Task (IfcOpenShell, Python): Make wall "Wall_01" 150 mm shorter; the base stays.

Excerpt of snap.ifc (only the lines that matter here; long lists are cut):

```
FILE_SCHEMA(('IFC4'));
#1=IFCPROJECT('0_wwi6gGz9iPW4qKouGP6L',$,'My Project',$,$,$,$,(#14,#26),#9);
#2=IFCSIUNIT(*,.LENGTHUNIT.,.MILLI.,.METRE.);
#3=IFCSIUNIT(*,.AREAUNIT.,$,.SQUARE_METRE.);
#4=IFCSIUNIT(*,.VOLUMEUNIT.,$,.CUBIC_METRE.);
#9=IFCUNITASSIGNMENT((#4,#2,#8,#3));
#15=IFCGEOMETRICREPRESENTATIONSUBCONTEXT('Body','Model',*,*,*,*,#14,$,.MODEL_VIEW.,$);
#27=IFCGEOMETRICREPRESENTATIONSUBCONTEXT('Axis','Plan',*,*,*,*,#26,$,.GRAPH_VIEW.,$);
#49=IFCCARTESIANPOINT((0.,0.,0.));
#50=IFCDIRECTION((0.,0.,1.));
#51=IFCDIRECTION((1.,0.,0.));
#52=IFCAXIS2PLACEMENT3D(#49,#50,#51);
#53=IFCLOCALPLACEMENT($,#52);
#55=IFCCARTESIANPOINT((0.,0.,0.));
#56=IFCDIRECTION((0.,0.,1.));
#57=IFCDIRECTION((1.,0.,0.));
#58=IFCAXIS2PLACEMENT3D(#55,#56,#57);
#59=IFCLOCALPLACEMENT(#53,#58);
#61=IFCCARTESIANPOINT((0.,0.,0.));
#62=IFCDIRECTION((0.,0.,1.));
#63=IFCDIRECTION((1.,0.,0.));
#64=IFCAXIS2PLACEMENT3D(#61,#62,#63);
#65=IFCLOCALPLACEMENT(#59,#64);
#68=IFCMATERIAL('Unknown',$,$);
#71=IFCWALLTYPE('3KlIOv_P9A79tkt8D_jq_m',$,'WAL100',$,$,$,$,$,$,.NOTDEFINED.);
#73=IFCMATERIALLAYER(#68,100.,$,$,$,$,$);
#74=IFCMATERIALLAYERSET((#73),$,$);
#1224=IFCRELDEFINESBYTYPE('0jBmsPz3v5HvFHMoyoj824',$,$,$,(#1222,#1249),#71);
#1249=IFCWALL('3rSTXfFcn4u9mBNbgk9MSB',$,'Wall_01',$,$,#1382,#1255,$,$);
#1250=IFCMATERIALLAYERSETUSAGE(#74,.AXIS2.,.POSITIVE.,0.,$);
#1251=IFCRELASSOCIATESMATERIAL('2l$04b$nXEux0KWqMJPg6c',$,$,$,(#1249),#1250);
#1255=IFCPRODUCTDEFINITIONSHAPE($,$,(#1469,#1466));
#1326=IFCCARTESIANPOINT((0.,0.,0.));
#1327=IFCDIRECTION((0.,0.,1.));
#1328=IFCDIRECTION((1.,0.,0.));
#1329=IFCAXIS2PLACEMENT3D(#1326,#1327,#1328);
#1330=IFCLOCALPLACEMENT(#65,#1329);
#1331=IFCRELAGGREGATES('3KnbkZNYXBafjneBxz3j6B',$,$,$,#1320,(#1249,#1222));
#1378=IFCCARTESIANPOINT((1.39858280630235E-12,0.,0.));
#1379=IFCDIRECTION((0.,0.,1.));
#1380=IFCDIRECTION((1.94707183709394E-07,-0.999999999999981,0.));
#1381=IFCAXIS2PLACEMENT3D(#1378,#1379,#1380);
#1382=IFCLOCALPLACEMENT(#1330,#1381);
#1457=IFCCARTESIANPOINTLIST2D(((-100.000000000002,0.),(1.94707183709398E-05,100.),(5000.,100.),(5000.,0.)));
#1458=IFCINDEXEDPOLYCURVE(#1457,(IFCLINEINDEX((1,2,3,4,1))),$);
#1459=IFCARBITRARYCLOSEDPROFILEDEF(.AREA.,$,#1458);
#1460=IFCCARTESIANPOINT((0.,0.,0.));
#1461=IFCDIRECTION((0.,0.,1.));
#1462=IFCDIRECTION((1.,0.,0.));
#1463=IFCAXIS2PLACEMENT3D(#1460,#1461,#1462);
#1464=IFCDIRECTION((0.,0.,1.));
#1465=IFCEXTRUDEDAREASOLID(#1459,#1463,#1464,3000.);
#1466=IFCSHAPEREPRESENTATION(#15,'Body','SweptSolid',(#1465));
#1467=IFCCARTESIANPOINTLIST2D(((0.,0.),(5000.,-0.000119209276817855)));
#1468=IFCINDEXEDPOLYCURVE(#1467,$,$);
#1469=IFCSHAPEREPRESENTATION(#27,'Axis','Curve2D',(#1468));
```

```python
import ifcopenshell
import ifcopenshell.geom
import ifcopenshell.util.representation
import ifcopenshell.util.shape
import ifcopenshell.util.unit

model = ifcopenshell.open("snap.ifc")
unit_scale = ifcopenshell.util.unit.calculate_unit_scale(model)
settings = ifcopenshell.geom.settings()


def volume(element):
    """Net volume in cubic metres, openings subtracted."""
    shape = ifcopenshell.geom.create_shape(settings, element)
    return ifcopenshell.util.shape.get_volume(shape.geometry)


wall = model.by_id(1249)
before = volume(wall)

body = ifcopenshell.util.representation.get_representation(wall, "Model", "Body")
solid = body.Items[0]
old_height = solid.Depth
solid.Depth -= 0.15 / unit_scale
after = volume(wall)

print(f"height {old_height:g} -> {solid.Depth:g}, volume {before:.3f} -> {after:.3f} m3")

model.write("snap_edited.ifc")
```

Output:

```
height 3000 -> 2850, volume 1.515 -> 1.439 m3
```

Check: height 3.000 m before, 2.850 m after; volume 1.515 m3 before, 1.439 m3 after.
